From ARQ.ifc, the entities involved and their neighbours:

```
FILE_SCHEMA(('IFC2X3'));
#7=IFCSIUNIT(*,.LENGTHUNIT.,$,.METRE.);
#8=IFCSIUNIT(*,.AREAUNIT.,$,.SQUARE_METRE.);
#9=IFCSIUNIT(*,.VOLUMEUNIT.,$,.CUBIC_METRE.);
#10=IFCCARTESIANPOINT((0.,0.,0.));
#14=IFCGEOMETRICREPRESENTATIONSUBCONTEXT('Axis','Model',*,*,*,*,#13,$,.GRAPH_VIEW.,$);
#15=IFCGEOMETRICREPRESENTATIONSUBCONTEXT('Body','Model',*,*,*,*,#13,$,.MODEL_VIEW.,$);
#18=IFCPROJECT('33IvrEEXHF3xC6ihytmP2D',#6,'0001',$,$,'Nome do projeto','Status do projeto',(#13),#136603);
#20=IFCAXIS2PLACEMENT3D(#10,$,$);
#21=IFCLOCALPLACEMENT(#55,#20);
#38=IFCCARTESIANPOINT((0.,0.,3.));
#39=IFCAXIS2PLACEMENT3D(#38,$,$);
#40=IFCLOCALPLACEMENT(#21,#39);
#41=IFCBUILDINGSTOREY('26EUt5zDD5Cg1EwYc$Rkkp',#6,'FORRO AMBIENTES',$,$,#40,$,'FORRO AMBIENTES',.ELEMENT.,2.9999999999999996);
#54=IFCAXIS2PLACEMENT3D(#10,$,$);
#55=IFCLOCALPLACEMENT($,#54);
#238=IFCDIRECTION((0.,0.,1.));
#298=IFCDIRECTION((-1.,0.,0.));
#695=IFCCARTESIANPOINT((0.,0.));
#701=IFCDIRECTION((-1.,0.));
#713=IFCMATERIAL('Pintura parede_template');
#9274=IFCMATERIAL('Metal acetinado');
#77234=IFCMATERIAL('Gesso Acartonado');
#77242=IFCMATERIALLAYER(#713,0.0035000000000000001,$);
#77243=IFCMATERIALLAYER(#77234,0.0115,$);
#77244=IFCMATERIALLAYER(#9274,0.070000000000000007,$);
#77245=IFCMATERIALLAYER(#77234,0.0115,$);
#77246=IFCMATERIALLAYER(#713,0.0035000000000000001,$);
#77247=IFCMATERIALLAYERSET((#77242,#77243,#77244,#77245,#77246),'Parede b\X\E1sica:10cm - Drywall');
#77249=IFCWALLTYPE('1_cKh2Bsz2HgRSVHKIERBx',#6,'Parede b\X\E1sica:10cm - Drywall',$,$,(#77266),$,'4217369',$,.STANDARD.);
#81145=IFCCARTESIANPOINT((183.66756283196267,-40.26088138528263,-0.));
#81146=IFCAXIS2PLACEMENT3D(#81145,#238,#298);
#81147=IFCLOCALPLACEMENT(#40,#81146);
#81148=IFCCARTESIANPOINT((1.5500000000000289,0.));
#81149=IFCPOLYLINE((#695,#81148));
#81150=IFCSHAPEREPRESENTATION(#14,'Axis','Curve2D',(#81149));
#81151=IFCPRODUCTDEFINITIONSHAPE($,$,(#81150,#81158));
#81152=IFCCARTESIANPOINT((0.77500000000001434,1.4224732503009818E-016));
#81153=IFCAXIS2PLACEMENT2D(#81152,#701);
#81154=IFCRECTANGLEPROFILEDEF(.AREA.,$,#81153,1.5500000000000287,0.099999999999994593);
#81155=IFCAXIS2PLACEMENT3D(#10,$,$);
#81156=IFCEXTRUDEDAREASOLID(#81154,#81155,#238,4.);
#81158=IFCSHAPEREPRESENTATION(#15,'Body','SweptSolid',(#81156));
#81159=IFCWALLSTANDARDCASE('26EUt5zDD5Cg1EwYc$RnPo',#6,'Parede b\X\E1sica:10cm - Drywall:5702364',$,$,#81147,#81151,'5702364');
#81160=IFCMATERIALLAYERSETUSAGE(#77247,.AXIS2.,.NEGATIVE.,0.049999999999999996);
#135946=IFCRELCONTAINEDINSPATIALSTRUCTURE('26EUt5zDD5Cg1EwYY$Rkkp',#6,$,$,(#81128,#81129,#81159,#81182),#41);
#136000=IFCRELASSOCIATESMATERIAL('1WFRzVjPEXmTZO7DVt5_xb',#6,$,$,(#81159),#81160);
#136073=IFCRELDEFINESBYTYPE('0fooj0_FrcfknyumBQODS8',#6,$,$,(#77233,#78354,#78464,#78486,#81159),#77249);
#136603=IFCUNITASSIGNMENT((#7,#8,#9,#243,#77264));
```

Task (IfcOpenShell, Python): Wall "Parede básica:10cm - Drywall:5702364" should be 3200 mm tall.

```python
import ifcopenshell
import ifcopenshell.geom
import ifcopenshell.util.representation
import ifcopenshell.util.shape
import ifcopenshell.util.unit

model = ifcopenshell.open("ARQ.ifc")
unit_scale = ifcopenshell.util.unit.calculate_unit_scale(model)
settings = ifcopenshell.geom.settings()


def volume(element):
    """Net volume in cubic metres, openings subtracted."""
    shape = ifcopenshell.geom.create_shape(settings, element)
    return ifcopenshell.util.shape.get_volume(shape.geometry)


wall = model.by_guid("26EUt5zDD5Cg1EwYc$RnPo")
before = volume(wall)

body = ifcopenshell.util.representation.get_representation(wall, "Model", "Body")
solid = body.Items[0]
old_height = solid.Depth
solid.Depth = 3.2 / unit_scale
after = volume(wall)

print(f"height {old_height:g} -> {solid.Depth:g}, volume {before:.3f} -> {after:.3f} m3")

model.write("ARQ_updated.ifc")
```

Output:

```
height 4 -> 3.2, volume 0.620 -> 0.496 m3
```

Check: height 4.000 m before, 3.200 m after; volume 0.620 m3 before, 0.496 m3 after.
